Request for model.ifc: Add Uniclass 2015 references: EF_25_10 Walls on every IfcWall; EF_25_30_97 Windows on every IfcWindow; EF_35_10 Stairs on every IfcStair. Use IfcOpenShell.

First a look at what the model holds.

```python
import ifcopenshell

model = ifcopenshell.open("model.ifc")
print(model.schema)
print("classifications:", [c.Name for c in model.by_type("IfcClassification")])
for ifc_class in ("IfcDoor", "IfcRoof", "IfcStair", "IfcWall", "IfcWindow"):
    print(ifc_class, len(model.by_type(ifc_class)))
```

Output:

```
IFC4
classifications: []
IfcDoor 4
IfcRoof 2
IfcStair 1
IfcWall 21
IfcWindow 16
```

```python
import ifcopenshell
import ifcopenshell.api.classification

model = ifcopenshell.open("model.ifc")

system = ifcopenshell.api.classification.add_classification(model, classification="Uniclass 2015")

codes = {
    "IfcWall": ("EF_25_10", "Walls"),
    "IfcWindow": ("EF_25_30_97", "Windows"),
    "IfcStair": ("EF_35_10", "Stairs"),
}
for ifc_class, (code, name) in codes.items():
    products = model.by_type(ifc_class)
    ifcopenshell.api.classification.add_reference(
        model, products=products, classification=system, identification=code, name=name
    )
    print(code, len(products))

model.write("model_edited.ifc")
```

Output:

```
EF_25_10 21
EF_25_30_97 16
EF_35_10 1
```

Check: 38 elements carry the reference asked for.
